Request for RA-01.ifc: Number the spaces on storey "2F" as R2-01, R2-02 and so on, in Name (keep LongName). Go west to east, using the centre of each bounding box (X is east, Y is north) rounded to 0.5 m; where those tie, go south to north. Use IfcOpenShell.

First a look at what the model holds.

```python
import ifcopenshell
import ifcopenshell.util.element
import ifcopenshell.util.placement

model = ifcopenshell.open("RA-01.ifc")
print(model.schema)
storey = next(s for s in model.by_type("IfcBuildingStorey") if s.Name == "2F")
spaces = [e for e in ifcopenshell.util.element.get_decomposition(storey) if e.is_a("IfcSpace")]
for e in sorted(spaces, key=lambda e: e.id()):
    origin = ifcopenshell.util.placement.get_local_placement(e.ObjectPlacement)[:3, 3]
    print(e.id(), e.Name, e.LongName, origin.round(2) + 0.0, sep=" | ")
```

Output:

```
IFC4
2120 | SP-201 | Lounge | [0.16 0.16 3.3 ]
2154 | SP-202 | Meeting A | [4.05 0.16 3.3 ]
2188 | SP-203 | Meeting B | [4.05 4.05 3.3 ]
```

```python
import ifcopenshell
import ifcopenshell.geom
import ifcopenshell.util.element
import ifcopenshell.util.shape

model = ifcopenshell.open("RA-01.ifc")
settings = ifcopenshell.geom.settings()
settings.set("use-world-coords", True)


def centre(element):
    shape = ifcopenshell.geom.create_shape(settings, element)
    return ifcopenshell.util.shape.get_bbox_centroid(shape.geometry)


storey = next(s for s in model.by_type("IfcBuildingStorey") if s.Name == "2F")
spaces = [e for e in ifcopenshell.util.element.get_decomposition(storey) if e.is_a("IfcSpace")]

# Insertion points can sit at a corner or the storey origin, so sort by the geometry (in metres).
centres = {e: centre(e) for e in spaces}
spaces.sort(key=lambda e: (round(centres[e][0] / 0.5), centres[e][1]))

for i, e in enumerate(spaces, start=1):
    number = f"R2-{i:02d}"
    e.Name = number
    print(e.id(), number)

model.write("RA-01-out.ifc")
```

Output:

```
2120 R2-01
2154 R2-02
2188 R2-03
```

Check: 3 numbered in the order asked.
